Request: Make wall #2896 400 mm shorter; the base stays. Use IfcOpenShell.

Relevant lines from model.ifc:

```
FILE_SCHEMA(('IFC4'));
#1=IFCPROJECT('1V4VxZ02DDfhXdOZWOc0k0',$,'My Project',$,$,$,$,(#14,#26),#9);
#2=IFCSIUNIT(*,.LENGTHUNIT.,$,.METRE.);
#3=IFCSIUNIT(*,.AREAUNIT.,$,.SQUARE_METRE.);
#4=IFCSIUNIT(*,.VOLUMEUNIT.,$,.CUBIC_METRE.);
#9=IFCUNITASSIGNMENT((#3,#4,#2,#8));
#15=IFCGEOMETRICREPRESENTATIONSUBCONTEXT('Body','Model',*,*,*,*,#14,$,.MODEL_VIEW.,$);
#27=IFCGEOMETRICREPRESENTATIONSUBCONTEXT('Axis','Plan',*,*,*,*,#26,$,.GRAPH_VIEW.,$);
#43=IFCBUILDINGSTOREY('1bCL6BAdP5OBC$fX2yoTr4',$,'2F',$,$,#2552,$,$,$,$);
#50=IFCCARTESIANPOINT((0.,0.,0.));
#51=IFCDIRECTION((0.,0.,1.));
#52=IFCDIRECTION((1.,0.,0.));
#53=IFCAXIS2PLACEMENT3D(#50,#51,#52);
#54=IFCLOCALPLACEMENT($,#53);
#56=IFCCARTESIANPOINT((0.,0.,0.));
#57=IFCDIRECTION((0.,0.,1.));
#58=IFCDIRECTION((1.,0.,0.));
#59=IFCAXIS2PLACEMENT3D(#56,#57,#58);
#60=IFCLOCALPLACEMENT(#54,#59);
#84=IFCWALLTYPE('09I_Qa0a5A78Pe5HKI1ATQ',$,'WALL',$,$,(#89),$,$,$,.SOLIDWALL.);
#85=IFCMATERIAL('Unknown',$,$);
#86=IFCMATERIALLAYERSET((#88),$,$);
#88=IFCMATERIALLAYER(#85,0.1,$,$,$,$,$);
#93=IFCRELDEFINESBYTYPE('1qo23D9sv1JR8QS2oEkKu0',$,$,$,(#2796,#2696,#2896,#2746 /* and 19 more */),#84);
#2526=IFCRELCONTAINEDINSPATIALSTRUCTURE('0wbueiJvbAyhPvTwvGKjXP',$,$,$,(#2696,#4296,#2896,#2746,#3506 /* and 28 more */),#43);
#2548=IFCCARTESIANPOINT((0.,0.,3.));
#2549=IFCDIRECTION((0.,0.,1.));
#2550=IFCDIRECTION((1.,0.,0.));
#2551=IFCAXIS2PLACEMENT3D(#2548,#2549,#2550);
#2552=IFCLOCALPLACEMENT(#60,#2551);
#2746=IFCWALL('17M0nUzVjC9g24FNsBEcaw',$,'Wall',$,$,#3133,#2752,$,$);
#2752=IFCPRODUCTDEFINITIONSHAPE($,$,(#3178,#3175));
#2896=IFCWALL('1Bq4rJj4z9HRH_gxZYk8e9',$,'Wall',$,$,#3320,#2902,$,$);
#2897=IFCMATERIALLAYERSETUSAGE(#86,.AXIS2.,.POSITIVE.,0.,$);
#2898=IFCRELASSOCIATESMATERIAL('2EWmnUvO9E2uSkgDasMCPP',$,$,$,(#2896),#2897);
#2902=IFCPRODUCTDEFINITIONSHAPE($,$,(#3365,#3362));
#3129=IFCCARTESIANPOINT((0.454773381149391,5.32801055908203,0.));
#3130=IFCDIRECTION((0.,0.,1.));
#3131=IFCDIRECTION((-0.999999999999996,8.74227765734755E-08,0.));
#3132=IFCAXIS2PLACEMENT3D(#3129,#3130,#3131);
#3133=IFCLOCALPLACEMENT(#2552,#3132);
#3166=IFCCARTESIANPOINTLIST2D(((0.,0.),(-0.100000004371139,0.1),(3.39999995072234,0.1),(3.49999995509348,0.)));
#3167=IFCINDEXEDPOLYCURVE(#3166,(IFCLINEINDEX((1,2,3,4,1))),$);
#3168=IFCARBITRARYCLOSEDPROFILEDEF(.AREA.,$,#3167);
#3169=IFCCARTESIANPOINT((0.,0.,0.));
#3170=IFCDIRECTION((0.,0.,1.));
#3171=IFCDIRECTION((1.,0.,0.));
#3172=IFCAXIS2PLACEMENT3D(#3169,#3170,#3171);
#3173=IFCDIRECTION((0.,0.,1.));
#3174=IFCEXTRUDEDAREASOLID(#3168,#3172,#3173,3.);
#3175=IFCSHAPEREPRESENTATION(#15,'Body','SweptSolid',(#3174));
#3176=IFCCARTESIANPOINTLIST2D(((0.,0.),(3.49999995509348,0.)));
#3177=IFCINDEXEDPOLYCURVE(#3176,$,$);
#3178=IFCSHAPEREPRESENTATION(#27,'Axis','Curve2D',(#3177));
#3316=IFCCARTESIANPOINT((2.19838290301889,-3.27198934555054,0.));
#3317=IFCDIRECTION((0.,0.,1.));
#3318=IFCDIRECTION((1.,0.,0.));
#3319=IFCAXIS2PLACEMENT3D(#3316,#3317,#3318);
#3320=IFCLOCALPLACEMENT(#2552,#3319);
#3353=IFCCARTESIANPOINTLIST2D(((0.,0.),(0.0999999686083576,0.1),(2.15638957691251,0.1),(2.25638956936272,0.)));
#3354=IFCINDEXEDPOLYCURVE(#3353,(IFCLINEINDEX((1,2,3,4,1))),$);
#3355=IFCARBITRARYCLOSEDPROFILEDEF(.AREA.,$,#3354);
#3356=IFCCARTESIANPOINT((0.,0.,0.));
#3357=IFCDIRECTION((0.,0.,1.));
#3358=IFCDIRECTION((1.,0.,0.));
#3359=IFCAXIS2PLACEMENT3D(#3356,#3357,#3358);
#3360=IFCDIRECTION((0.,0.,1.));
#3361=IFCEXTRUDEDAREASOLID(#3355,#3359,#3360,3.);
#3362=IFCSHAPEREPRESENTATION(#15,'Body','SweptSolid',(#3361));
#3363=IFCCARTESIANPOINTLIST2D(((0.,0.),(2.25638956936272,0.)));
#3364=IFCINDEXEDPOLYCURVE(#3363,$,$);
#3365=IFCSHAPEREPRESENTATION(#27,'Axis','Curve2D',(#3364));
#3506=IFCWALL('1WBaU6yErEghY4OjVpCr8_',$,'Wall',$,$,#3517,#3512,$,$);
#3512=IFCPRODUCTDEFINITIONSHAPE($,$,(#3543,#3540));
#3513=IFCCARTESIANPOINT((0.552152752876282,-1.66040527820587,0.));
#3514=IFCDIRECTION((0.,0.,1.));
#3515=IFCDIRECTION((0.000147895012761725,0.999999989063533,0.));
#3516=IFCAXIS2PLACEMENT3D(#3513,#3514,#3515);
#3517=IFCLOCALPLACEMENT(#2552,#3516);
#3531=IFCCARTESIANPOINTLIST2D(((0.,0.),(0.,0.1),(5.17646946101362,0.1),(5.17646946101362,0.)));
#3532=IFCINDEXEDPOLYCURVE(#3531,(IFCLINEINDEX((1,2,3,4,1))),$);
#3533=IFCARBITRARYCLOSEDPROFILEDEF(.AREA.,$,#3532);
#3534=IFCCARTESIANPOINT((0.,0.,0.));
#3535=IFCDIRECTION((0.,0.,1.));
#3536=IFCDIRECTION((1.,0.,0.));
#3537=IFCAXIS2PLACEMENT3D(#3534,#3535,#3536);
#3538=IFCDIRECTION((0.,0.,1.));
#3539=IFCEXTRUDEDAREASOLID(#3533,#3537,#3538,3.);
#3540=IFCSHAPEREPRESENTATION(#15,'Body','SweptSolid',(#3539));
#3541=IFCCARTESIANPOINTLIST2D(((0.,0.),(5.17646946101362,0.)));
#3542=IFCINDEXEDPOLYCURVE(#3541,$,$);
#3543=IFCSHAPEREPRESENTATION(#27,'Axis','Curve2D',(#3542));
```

```python
import ifcopenshell
import ifcopenshell.geom
import ifcopenshell.util.representation
import ifcopenshell.util.shape

model = ifcopenshell.open("model.ifc")
settings = ifcopenshell.geom.settings()


def volume(element):
    """Net volume in cubic metres, openings subtracted."""
    shape = ifcopenshell.geom.create_shape(settings, element)
    return ifcopenshell.util.shape.get_volume(shape.geometry)


wall = model.by_guid("1Bq4rJj4z9HRH_gxZYk8e9")
before = volume(wall)

body = ifcopenshell.util.representation.get_representation(wall, "Model", "Body")
solid = body.Items[0]
old_height = solid.Depth
solid.Depth -= 0.4
after = volume(wall)

print(f"height {old_height:g} -> {solid.Depth:g}, volume {before:.3f} -> {after:.3f} m3")

model.write("model_v2.ifc")
```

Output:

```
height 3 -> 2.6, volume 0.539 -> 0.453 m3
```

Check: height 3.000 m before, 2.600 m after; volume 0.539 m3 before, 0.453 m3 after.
